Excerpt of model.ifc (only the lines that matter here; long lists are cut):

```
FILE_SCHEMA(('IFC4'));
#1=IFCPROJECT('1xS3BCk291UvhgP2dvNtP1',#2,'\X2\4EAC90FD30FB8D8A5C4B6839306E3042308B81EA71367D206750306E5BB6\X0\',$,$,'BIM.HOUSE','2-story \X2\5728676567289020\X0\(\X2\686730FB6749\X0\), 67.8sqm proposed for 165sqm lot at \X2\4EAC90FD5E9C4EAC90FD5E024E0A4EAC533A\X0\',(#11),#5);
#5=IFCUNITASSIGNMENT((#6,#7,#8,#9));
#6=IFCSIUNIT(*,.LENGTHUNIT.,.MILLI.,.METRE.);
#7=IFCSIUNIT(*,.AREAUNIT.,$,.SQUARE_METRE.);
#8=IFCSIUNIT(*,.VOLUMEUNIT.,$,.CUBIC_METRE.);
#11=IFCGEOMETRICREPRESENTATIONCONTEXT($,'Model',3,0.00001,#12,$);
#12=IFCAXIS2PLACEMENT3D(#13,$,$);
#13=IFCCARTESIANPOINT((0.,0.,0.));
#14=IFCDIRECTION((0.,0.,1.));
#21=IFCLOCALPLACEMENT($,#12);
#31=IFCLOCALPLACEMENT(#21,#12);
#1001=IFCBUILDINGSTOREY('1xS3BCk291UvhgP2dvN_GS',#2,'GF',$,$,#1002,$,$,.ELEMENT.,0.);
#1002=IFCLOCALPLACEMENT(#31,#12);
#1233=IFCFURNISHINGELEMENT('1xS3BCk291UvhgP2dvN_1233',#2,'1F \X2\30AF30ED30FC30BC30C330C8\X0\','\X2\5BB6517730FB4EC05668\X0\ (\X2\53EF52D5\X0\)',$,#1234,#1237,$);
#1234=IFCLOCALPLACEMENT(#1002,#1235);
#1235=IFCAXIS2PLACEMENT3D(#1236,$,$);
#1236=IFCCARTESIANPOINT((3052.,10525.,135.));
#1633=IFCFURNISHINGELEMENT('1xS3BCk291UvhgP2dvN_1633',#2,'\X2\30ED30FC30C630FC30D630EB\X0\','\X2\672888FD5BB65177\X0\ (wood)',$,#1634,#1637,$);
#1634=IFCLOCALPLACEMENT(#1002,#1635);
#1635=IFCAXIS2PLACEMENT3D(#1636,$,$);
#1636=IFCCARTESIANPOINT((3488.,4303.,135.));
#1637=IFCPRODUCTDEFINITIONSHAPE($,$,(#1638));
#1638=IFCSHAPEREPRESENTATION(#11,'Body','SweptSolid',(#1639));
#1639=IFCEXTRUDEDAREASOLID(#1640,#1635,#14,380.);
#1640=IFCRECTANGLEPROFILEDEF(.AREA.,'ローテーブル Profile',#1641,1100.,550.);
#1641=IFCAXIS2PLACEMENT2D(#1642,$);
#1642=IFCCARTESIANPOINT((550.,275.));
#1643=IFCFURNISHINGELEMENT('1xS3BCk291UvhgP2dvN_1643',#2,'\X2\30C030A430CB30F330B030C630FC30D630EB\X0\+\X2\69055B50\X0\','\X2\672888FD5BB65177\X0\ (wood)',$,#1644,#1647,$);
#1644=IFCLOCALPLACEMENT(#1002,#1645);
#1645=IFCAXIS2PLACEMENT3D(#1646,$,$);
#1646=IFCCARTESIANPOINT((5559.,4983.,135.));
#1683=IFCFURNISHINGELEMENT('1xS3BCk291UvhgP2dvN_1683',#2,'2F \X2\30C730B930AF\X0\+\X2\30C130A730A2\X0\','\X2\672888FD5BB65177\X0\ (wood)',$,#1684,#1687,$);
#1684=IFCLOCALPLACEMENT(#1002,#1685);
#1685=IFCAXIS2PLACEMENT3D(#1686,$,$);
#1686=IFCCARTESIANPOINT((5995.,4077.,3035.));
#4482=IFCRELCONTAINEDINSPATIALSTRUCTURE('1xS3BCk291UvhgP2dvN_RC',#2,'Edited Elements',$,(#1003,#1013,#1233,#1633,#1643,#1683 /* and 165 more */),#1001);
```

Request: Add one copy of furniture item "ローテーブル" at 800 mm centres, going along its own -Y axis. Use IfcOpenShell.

```python
import ifcopenshell
import ifcopenshell.api.geometry
import ifcopenshell.api.root
import ifcopenshell.util.element
import ifcopenshell.util.placement
import ifcopenshell.util.unit

model = ifcopenshell.open("model.ifc")
unit_scale = ifcopenshell.util.unit.calculate_unit_scale(model)


def reuse_history(source, copy):
    """copy_class also copies each property set's owner history, people and application; keep the originals."""
    for rel in copy.IsDefinedBy:
        if rel.is_a("IfcRelDefinesByProperties") and (history := rel.RelatingPropertyDefinition.OwnerHistory):
            rel.RelatingPropertyDefinition.OwnerHistory = source.OwnerHistory
            ifcopenshell.util.element.remove_deep2(model, history)


source = model.by_guid("1xS3BCk291UvhgP2dvN_1633")
base = ifcopenshell.util.placement.get_local_placement(source.ObjectPlacement)
step = -base[:3, 1] * 0.8 / unit_scale

for i in range(1, 2):
    copy = ifcopenshell.api.root.copy_class(model, product=source)
    copy.Representation = ifcopenshell.util.element.copy_deep(
        model, source.Representation, exclude=["IfcGeometricRepresentationContext", "IfcRepresentationMap"]
    )
    reuse_history(source, copy)
    matrix = base.copy()
    matrix[:3, 3] += i * step
    print("added at", matrix[:3, 3].round(3) + 0.0)
    ifcopenshell.api.geometry.edit_object_placement(model, product=copy, matrix=matrix, is_si=False)

model.write("model_edited.ifc")
```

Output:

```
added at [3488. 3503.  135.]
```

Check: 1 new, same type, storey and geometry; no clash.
